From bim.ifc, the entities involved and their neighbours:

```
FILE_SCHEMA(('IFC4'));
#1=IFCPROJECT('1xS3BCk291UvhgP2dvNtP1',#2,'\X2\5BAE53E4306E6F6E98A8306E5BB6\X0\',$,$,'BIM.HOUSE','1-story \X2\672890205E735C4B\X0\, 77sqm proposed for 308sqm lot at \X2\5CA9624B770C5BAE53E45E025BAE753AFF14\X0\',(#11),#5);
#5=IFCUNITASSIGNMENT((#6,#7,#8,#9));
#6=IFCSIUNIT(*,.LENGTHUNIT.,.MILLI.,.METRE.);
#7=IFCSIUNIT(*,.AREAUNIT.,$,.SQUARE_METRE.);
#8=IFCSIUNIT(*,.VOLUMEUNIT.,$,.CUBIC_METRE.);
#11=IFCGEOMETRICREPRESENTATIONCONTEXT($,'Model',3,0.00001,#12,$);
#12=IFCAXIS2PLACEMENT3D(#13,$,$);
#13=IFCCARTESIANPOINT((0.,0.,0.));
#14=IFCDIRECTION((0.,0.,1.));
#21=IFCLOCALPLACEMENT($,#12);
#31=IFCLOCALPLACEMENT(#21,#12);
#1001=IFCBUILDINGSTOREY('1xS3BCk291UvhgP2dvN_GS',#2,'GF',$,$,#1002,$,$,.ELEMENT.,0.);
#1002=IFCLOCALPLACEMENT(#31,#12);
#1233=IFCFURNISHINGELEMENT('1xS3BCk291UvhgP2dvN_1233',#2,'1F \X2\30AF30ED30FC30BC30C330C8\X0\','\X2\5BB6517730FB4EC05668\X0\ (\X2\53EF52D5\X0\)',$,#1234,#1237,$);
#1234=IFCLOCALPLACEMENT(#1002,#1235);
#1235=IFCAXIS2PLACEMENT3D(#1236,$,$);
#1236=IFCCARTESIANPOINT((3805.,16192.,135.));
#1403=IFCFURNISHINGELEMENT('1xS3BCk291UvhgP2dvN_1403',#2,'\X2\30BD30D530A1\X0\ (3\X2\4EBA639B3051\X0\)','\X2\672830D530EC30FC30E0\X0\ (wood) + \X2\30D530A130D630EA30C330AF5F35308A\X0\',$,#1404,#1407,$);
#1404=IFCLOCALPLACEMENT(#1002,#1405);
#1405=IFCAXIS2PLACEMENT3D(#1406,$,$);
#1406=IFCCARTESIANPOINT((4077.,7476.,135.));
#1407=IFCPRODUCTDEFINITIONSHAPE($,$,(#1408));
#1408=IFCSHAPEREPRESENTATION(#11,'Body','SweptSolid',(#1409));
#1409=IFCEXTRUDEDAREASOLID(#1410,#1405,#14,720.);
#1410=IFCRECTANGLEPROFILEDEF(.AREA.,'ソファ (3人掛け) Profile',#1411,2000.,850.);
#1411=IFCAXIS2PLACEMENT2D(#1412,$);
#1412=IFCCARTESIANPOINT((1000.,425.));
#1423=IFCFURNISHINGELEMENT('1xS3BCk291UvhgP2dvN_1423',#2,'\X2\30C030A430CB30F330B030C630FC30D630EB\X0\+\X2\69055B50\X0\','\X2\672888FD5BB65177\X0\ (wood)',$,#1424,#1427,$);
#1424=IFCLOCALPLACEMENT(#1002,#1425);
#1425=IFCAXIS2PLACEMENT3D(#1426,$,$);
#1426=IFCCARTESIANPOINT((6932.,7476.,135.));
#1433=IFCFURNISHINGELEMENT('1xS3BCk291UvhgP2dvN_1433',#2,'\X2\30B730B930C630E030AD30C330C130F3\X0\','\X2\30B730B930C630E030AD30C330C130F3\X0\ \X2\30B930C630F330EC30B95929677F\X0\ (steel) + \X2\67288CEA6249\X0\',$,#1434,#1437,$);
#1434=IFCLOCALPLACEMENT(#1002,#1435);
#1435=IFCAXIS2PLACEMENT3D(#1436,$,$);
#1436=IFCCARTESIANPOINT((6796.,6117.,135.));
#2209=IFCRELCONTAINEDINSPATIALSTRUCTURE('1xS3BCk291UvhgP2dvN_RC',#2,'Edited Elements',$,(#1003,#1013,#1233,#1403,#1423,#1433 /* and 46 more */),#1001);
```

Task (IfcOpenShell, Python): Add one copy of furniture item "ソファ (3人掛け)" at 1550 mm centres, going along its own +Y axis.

```python
import ifcopenshell
import ifcopenshell.api.geometry
import ifcopenshell.api.root
import ifcopenshell.util.element
import ifcopenshell.util.placement

model = ifcopenshell.open("bim.ifc")


def reuse_history(source, copy):
    """copy_class also copies each property set's owner history, people and application; keep the originals."""
    for rel in copy.IsDefinedBy:
        if rel.is_a("IfcRelDefinesByProperties") and (history := rel.RelatingPropertyDefinition.OwnerHistory):
            rel.RelatingPropertyDefinition.OwnerHistory = source.OwnerHistory
            ifcopenshell.util.element.remove_deep2(model, history)


source = model.by_guid("1xS3BCk291UvhgP2dvN_1403")
base = ifcopenshell.util.placement.get_local_placement(source.ObjectPlacement)
step = base[:3, 1] * 1550.0

for i in range(1, 2):
    copy = ifcopenshell.api.root.copy_class(model, product=source)
    copy.Representation = ifcopenshell.util.element.copy_deep(
        model, source.Representation, exclude=["IfcGeometricRepresentationContext", "IfcRepresentationMap"]
    )
    reuse_history(source, copy)
    matrix = base.copy()
    matrix[:3, 3] += i * step
    print("added at", matrix[:3, 3].round(3) + 0.0)
    ifcopenshell.api.geometry.edit_object_placement(model, product=copy, matrix=matrix, is_si=False)

model.write("bim_edited.ifc")
```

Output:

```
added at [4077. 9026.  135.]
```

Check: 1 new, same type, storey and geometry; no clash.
